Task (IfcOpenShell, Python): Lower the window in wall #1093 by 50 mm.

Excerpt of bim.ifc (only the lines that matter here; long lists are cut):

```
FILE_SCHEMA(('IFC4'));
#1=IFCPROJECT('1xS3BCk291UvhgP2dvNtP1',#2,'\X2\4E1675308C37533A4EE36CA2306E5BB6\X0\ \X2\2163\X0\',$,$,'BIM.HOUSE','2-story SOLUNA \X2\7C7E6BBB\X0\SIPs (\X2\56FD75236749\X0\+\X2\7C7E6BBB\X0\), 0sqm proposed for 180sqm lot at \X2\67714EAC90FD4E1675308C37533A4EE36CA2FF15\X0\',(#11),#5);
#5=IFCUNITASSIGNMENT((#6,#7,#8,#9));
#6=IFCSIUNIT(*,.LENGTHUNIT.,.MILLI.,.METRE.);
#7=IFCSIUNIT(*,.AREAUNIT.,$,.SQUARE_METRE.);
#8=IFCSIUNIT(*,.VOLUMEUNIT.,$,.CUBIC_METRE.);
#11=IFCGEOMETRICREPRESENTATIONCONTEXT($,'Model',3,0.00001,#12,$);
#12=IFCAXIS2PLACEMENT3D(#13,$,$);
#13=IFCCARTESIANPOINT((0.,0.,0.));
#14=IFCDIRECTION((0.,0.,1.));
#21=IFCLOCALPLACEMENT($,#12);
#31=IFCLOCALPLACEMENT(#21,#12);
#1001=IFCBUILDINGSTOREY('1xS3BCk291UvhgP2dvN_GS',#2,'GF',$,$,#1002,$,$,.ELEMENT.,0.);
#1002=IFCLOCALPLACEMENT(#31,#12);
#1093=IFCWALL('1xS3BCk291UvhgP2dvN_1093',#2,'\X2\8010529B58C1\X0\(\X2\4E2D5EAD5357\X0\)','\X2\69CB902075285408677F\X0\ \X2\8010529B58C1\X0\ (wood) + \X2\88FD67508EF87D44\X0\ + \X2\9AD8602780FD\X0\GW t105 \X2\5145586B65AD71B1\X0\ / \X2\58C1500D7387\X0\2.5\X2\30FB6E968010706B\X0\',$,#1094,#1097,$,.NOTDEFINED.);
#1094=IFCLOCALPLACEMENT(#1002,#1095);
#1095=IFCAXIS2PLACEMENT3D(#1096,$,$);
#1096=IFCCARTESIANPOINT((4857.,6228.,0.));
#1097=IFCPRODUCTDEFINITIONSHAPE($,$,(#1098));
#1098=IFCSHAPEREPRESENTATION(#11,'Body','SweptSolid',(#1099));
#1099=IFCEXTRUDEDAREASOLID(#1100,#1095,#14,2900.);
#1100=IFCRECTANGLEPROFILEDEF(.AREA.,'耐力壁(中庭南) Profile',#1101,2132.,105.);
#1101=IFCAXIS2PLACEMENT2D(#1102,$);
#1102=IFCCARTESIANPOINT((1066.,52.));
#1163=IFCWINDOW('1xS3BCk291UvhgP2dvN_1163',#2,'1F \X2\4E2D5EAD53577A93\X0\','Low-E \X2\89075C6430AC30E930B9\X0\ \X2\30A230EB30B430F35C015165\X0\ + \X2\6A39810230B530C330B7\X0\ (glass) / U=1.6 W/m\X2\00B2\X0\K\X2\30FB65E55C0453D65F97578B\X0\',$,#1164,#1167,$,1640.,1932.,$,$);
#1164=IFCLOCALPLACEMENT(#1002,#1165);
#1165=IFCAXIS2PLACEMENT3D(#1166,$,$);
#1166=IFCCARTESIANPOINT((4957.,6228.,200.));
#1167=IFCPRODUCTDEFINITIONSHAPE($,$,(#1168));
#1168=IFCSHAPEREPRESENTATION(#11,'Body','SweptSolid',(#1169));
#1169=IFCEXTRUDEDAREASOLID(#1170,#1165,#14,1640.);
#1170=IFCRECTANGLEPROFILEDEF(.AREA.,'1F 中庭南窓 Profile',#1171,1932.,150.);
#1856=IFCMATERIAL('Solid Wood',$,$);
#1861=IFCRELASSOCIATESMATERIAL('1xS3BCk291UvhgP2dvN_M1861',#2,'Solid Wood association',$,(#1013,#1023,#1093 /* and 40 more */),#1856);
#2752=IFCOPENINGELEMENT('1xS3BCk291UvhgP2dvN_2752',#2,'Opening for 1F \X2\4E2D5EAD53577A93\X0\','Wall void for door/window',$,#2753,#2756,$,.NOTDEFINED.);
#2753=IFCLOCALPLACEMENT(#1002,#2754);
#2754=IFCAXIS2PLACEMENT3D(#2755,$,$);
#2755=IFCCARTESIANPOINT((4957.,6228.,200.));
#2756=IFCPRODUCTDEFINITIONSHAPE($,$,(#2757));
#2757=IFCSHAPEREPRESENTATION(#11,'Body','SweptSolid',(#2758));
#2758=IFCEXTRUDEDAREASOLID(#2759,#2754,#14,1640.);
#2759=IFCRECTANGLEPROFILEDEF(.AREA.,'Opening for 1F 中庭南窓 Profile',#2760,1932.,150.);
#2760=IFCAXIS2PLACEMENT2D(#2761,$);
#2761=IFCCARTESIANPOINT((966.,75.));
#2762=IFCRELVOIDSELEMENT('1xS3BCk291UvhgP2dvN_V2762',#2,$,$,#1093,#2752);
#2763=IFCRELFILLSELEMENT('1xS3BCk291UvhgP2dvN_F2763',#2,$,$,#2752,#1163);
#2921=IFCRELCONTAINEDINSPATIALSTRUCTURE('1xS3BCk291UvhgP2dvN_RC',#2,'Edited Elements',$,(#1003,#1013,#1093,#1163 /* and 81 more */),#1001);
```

```python
import numpy as np
import ifcopenshell
import ifcopenshell.api.geometry
import ifcopenshell.util.placement
import ifcopenshell.util.unit

model = ifcopenshell.open("bim.ifc")
unit_scale = ifcopenshell.util.unit.calculate_unit_scale(model)

window = model.by_guid("1xS3BCk291UvhgP2dvN_1163")
opening = window.FillsVoids[0].RelatingOpeningElement
dz = -0.05 / unit_scale

shift = np.array([0.0, 0.0, dz])
# The window is not placed relative to its opening, so move both.
for product in (opening, window):
    matrix = ifcopenshell.util.placement.get_local_placement(product.ObjectPlacement)
    matrix[:3, 3] += shift
    ifcopenshell.api.geometry.edit_object_placement(model, product=product, matrix=matrix, is_si=False)

print(f"moved by {dz * unit_scale:+.3f} m")

model.write("bim_edited.ifc")
```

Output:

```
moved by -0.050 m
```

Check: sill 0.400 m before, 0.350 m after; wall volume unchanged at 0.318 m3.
